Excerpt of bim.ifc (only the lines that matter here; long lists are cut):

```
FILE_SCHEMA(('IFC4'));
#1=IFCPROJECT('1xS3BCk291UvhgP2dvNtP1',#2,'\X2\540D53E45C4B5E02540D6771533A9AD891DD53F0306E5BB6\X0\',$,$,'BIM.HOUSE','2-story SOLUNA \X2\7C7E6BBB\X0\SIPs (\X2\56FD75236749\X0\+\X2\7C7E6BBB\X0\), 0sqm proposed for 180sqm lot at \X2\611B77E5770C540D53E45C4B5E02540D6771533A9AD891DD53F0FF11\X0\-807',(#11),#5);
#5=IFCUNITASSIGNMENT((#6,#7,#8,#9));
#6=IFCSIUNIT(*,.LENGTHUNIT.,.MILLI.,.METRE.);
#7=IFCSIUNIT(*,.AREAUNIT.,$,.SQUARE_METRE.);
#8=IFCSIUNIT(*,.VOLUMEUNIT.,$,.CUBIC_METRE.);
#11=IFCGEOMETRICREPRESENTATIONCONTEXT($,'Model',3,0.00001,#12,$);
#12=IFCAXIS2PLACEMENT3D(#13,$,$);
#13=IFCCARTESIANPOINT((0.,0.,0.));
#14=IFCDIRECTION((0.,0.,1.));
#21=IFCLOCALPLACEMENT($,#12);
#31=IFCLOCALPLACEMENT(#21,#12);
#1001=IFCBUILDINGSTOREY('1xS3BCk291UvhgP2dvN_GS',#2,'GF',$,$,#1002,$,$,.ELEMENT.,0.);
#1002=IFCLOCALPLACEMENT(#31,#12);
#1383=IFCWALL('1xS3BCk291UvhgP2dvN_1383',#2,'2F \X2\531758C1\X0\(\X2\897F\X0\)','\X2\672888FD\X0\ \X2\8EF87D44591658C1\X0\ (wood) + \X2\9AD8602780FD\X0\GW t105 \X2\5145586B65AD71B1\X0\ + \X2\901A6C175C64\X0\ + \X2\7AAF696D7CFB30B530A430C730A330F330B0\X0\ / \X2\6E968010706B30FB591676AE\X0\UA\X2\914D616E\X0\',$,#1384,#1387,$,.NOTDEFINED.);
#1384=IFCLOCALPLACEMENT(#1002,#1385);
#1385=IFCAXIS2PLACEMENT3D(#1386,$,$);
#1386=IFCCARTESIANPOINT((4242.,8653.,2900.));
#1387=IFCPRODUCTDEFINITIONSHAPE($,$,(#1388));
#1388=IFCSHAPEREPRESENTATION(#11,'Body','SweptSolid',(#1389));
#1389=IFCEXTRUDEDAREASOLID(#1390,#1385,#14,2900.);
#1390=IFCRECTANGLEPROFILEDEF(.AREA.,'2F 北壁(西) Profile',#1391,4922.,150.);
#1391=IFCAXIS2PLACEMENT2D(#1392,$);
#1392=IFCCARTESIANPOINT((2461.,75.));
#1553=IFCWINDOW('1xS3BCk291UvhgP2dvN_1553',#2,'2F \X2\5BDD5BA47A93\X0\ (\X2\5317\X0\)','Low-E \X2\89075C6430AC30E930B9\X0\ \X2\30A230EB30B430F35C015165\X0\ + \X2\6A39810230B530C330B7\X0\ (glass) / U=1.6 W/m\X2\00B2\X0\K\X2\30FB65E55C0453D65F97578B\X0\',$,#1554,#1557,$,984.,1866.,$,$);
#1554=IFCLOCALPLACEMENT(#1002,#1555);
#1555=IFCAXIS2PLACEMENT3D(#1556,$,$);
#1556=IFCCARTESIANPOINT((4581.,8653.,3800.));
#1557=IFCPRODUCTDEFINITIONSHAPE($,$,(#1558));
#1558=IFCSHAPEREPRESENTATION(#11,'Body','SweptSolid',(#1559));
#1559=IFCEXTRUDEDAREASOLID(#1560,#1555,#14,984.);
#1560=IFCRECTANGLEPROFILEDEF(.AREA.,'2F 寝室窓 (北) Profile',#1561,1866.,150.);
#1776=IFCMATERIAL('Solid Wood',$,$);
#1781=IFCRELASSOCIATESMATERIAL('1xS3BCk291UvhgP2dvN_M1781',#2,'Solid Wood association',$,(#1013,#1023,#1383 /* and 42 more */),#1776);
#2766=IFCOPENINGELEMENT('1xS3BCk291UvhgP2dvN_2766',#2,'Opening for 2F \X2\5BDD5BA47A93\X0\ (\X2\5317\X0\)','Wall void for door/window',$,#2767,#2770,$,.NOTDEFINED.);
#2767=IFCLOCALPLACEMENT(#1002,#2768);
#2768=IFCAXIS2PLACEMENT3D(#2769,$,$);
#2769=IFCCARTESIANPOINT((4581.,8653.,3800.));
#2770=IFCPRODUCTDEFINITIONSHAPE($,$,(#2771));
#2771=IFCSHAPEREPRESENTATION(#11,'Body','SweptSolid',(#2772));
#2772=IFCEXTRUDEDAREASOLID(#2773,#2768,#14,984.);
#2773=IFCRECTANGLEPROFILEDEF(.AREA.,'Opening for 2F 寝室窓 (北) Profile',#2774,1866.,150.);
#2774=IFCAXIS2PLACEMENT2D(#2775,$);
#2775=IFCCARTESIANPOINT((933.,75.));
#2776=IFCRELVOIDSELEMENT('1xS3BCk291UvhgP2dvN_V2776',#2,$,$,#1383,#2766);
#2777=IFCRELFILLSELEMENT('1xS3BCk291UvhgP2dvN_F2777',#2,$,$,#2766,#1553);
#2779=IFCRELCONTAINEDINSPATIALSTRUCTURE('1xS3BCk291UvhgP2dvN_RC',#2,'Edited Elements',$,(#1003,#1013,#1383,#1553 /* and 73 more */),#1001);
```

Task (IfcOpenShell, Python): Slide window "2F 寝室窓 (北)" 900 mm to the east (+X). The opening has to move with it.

```python
import ifcopenshell
import ifcopenshell.api.geometry
import ifcopenshell.util.placement

model = ifcopenshell.open("bim.ifc")

window = model.by_guid("1xS3BCk291UvhgP2dvN_1553")
opening = window.FillsVoids[0].RelatingOpeningElement
wall = opening.VoidsElements[0].RelatingBuildingElement

wall_matrix = ifcopenshell.util.placement.get_local_placement(wall.ObjectPlacement)
shift = wall_matrix[:3, 0] * 900.0
before = ifcopenshell.util.placement.get_local_placement(window.ObjectPlacement)[:3, 3].copy()

# The window is not placed relative to its opening, so move both.
for product in (opening, window):
    matrix = ifcopenshell.util.placement.get_local_placement(product.ObjectPlacement)
    matrix[:3, 3] += shift
    ifcopenshell.api.geometry.edit_object_placement(model, product=product, matrix=matrix, is_si=False)

after = ifcopenshell.util.placement.get_local_placement(window.ObjectPlacement)[:3, 3]
print("window moved by", (after - before).round(3) + 0.0)

model.write("bim_edited.ifc")
```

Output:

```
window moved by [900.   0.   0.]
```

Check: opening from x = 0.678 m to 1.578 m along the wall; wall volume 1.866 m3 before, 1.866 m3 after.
